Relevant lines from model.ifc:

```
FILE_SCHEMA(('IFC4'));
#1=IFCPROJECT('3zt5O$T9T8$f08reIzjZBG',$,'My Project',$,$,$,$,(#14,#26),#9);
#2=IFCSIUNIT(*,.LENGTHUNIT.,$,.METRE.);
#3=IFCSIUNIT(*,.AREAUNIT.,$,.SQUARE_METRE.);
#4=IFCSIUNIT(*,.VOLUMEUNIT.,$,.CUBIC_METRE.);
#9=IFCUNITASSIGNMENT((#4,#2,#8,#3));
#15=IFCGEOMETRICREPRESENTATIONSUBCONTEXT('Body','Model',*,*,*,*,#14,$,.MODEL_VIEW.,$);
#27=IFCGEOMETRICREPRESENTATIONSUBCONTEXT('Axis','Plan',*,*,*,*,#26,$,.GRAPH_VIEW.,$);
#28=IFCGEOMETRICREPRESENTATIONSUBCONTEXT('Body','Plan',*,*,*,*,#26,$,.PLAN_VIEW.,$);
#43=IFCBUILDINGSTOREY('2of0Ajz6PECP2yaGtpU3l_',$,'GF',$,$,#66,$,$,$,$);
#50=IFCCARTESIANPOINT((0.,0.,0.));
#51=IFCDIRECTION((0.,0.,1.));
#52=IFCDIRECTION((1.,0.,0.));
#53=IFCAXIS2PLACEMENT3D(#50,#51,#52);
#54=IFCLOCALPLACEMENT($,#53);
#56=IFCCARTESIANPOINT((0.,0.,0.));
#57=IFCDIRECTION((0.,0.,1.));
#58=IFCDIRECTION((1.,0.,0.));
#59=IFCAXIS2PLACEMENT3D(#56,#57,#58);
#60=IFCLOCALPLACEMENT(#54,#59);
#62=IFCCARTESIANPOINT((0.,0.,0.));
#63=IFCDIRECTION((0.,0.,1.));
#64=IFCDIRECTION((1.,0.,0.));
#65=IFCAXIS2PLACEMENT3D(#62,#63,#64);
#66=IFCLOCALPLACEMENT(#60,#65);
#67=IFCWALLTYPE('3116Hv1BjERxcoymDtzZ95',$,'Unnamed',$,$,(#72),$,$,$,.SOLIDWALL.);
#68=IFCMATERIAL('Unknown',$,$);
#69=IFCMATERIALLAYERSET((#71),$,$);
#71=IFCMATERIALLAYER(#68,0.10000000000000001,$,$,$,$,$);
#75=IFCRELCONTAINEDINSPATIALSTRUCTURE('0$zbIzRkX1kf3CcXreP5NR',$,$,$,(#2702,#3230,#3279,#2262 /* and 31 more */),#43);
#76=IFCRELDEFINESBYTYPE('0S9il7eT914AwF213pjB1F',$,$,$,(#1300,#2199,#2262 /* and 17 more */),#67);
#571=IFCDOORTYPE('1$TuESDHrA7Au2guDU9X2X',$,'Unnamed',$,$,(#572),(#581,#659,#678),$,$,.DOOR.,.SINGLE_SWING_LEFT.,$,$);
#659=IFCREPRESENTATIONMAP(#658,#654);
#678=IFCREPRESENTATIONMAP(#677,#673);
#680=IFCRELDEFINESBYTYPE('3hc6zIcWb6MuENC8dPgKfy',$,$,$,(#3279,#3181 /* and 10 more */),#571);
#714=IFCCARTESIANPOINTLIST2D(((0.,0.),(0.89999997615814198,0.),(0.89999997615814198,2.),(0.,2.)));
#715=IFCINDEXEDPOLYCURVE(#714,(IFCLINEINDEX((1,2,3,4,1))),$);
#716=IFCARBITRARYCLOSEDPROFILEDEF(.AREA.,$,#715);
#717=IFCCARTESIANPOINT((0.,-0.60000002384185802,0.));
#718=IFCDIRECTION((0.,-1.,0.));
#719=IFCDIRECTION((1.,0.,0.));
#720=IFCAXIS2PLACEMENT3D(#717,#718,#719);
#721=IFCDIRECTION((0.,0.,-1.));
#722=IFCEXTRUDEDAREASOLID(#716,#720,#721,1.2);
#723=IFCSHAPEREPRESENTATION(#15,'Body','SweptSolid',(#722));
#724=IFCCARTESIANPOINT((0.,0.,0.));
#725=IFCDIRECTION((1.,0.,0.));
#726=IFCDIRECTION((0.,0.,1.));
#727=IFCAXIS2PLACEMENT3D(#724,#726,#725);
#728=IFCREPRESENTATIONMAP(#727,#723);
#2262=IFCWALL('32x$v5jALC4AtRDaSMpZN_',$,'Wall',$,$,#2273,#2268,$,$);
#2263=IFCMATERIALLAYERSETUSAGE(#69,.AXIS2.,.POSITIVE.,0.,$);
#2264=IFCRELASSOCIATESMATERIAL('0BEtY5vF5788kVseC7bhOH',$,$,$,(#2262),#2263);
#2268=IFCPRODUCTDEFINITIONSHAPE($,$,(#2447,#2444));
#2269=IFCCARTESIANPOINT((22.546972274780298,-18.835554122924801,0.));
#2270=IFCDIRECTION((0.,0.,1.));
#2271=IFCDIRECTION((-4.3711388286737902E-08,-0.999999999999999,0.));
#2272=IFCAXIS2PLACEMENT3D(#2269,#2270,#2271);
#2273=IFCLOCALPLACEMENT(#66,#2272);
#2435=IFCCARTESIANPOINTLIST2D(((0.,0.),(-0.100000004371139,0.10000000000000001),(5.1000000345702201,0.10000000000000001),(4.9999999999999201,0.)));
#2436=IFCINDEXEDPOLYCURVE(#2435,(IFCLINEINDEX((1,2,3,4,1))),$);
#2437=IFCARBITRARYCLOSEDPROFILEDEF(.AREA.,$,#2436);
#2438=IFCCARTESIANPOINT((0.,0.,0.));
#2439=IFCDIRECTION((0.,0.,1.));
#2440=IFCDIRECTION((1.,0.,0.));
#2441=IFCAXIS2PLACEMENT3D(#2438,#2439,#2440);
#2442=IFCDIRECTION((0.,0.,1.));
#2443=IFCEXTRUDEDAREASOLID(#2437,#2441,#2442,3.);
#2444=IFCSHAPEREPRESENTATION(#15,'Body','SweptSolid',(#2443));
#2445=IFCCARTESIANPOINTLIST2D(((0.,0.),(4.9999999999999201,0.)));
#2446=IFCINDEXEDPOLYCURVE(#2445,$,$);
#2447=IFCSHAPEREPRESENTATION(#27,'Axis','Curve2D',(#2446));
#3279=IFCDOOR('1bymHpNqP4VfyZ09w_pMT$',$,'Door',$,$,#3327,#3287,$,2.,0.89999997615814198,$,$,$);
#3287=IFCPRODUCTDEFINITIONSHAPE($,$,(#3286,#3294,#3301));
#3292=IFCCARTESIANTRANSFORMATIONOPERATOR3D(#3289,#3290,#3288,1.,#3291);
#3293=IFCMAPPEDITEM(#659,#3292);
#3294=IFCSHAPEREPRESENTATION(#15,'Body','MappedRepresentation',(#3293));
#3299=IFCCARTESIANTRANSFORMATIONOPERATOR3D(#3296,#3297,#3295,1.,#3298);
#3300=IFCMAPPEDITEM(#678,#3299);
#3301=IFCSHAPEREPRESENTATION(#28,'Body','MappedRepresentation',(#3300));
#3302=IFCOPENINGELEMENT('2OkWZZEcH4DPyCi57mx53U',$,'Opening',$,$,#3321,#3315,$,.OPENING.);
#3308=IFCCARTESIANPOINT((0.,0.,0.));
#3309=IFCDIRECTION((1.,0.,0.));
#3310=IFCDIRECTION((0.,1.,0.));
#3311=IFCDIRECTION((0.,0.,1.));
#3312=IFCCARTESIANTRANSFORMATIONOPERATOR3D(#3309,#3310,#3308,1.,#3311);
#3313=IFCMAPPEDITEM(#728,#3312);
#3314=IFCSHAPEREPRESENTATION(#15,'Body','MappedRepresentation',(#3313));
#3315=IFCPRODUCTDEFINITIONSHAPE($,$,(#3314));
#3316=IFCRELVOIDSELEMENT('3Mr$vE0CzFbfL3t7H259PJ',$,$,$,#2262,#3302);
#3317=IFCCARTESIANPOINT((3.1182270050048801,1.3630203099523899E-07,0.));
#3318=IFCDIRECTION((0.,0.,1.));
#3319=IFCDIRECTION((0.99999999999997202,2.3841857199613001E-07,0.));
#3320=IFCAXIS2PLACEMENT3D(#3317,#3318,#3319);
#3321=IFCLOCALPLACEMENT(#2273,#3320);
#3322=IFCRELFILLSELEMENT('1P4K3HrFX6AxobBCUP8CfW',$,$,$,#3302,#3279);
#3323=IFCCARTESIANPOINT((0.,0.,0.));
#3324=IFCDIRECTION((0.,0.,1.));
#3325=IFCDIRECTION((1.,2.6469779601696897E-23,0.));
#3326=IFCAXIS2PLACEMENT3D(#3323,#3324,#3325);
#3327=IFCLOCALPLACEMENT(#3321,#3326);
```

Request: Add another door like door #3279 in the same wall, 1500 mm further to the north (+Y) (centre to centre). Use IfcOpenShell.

```python
import ifcopenshell
import ifcopenshell.api.feature
import ifcopenshell.api.geometry
import ifcopenshell.api.root
import ifcopenshell.geom
import ifcopenshell.util.element
import ifcopenshell.util.placement
import ifcopenshell.util.shape

model = ifcopenshell.open("model.ifc")
settings = ifcopenshell.geom.settings()


def volume(element):
    """Net volume in cubic metres, openings subtracted."""
    shape = ifcopenshell.geom.create_shape(settings, element)
    return ifcopenshell.util.shape.get_volume(shape.geometry)


door = model.by_guid("1bymHpNqP4VfyZ09w_pMT$")
opening = door.FillsVoids[0].RelatingOpeningElement
wall = opening.VoidsElements[0].RelatingBuildingElement
before = volume(wall)
shift = ifcopenshell.util.placement.get_local_placement(wall.ObjectPlacement)[:3, 0] * -1.5

# copy_class copies the void relationship, type, container and properties, but no geometry.
new_opening = ifcopenshell.api.root.copy_class(model, product=opening)
new_opening.Representation = ifcopenshell.util.element.copy_deep(
    model, opening.Representation, exclude=["IfcGeometricRepresentationContext", "IfcRepresentationMap"]
)
new_door = ifcopenshell.api.root.copy_class(model, product=door)
new_door.Representation = ifcopenshell.util.element.copy_deep(
    model, door.Representation, exclude=["IfcGeometricRepresentationContext", "IfcRepresentationMap"]
)
ifcopenshell.api.feature.add_filling(model, opening=new_opening, element=new_door)

for old, new in ((opening, new_opening), (door, new_door)):
    matrix = ifcopenshell.util.placement.get_local_placement(old.ObjectPlacement)
    matrix[:3, 3] += shift
    ifcopenshell.api.geometry.edit_object_placement(model, product=new, matrix=matrix, is_si=False)

after = volume(wall)

print(f"wall volume {before:.3f} -> {after:.3f} m3")

model.write("model_updated.ifc")
```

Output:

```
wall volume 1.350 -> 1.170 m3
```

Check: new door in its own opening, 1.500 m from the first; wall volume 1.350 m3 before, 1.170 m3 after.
